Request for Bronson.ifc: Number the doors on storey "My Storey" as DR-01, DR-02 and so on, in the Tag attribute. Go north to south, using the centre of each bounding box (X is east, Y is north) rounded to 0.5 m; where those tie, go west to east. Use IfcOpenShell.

First a look at what the model holds.

```python
import ifcopenshell
import ifcopenshell.util.element
import ifcopenshell.util.placement

model = ifcopenshell.open("Bronson.ifc")
print(model.schema)
storey = next(s for s in model.by_type("IfcBuildingStorey") if s.Name == "My Storey")
doors = [e for e in ifcopenshell.util.element.get_decomposition(storey) if e.is_a("IfcDoor")]
for e in sorted(doors, key=lambda e: e.id()):
    origin = ifcopenshell.util.placement.get_local_placement(e.ObjectPlacement)[:3, 3]
    print(e.id(), e.Tag, e.Name, origin.round(2) + 0.0, sep=" | ")
```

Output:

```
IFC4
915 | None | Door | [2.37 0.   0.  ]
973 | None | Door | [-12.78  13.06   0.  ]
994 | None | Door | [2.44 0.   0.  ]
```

```python
import ifcopenshell
import ifcopenshell.geom
import ifcopenshell.util.element
import ifcopenshell.util.shape

model = ifcopenshell.open("Bronson.ifc")
settings = ifcopenshell.geom.settings()
settings.set("use-world-coords", True)


def centre(element):
    shape = ifcopenshell.geom.create_shape(settings, element)
    return ifcopenshell.util.shape.get_bbox_centroid(shape.geometry)


storey = next(s for s in model.by_type("IfcBuildingStorey") if s.Name == "My Storey")
doors = [e for e in ifcopenshell.util.element.get_decomposition(storey) if e.is_a("IfcDoor")]

# Insertion points can sit at a corner or the storey origin, so sort by the geometry (in metres).
centres = {e: centre(e) for e in doors}
doors.sort(key=lambda e: (-round(centres[e][1] / 0.5), centres[e][0]))

for i, e in enumerate(doors, start=1):
    number = f"DR-{i:02d}"
    e.Tag = number
    print(e.id(), number)

model.write("Bronson_edited.ifc")
```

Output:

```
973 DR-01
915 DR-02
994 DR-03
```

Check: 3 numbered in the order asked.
